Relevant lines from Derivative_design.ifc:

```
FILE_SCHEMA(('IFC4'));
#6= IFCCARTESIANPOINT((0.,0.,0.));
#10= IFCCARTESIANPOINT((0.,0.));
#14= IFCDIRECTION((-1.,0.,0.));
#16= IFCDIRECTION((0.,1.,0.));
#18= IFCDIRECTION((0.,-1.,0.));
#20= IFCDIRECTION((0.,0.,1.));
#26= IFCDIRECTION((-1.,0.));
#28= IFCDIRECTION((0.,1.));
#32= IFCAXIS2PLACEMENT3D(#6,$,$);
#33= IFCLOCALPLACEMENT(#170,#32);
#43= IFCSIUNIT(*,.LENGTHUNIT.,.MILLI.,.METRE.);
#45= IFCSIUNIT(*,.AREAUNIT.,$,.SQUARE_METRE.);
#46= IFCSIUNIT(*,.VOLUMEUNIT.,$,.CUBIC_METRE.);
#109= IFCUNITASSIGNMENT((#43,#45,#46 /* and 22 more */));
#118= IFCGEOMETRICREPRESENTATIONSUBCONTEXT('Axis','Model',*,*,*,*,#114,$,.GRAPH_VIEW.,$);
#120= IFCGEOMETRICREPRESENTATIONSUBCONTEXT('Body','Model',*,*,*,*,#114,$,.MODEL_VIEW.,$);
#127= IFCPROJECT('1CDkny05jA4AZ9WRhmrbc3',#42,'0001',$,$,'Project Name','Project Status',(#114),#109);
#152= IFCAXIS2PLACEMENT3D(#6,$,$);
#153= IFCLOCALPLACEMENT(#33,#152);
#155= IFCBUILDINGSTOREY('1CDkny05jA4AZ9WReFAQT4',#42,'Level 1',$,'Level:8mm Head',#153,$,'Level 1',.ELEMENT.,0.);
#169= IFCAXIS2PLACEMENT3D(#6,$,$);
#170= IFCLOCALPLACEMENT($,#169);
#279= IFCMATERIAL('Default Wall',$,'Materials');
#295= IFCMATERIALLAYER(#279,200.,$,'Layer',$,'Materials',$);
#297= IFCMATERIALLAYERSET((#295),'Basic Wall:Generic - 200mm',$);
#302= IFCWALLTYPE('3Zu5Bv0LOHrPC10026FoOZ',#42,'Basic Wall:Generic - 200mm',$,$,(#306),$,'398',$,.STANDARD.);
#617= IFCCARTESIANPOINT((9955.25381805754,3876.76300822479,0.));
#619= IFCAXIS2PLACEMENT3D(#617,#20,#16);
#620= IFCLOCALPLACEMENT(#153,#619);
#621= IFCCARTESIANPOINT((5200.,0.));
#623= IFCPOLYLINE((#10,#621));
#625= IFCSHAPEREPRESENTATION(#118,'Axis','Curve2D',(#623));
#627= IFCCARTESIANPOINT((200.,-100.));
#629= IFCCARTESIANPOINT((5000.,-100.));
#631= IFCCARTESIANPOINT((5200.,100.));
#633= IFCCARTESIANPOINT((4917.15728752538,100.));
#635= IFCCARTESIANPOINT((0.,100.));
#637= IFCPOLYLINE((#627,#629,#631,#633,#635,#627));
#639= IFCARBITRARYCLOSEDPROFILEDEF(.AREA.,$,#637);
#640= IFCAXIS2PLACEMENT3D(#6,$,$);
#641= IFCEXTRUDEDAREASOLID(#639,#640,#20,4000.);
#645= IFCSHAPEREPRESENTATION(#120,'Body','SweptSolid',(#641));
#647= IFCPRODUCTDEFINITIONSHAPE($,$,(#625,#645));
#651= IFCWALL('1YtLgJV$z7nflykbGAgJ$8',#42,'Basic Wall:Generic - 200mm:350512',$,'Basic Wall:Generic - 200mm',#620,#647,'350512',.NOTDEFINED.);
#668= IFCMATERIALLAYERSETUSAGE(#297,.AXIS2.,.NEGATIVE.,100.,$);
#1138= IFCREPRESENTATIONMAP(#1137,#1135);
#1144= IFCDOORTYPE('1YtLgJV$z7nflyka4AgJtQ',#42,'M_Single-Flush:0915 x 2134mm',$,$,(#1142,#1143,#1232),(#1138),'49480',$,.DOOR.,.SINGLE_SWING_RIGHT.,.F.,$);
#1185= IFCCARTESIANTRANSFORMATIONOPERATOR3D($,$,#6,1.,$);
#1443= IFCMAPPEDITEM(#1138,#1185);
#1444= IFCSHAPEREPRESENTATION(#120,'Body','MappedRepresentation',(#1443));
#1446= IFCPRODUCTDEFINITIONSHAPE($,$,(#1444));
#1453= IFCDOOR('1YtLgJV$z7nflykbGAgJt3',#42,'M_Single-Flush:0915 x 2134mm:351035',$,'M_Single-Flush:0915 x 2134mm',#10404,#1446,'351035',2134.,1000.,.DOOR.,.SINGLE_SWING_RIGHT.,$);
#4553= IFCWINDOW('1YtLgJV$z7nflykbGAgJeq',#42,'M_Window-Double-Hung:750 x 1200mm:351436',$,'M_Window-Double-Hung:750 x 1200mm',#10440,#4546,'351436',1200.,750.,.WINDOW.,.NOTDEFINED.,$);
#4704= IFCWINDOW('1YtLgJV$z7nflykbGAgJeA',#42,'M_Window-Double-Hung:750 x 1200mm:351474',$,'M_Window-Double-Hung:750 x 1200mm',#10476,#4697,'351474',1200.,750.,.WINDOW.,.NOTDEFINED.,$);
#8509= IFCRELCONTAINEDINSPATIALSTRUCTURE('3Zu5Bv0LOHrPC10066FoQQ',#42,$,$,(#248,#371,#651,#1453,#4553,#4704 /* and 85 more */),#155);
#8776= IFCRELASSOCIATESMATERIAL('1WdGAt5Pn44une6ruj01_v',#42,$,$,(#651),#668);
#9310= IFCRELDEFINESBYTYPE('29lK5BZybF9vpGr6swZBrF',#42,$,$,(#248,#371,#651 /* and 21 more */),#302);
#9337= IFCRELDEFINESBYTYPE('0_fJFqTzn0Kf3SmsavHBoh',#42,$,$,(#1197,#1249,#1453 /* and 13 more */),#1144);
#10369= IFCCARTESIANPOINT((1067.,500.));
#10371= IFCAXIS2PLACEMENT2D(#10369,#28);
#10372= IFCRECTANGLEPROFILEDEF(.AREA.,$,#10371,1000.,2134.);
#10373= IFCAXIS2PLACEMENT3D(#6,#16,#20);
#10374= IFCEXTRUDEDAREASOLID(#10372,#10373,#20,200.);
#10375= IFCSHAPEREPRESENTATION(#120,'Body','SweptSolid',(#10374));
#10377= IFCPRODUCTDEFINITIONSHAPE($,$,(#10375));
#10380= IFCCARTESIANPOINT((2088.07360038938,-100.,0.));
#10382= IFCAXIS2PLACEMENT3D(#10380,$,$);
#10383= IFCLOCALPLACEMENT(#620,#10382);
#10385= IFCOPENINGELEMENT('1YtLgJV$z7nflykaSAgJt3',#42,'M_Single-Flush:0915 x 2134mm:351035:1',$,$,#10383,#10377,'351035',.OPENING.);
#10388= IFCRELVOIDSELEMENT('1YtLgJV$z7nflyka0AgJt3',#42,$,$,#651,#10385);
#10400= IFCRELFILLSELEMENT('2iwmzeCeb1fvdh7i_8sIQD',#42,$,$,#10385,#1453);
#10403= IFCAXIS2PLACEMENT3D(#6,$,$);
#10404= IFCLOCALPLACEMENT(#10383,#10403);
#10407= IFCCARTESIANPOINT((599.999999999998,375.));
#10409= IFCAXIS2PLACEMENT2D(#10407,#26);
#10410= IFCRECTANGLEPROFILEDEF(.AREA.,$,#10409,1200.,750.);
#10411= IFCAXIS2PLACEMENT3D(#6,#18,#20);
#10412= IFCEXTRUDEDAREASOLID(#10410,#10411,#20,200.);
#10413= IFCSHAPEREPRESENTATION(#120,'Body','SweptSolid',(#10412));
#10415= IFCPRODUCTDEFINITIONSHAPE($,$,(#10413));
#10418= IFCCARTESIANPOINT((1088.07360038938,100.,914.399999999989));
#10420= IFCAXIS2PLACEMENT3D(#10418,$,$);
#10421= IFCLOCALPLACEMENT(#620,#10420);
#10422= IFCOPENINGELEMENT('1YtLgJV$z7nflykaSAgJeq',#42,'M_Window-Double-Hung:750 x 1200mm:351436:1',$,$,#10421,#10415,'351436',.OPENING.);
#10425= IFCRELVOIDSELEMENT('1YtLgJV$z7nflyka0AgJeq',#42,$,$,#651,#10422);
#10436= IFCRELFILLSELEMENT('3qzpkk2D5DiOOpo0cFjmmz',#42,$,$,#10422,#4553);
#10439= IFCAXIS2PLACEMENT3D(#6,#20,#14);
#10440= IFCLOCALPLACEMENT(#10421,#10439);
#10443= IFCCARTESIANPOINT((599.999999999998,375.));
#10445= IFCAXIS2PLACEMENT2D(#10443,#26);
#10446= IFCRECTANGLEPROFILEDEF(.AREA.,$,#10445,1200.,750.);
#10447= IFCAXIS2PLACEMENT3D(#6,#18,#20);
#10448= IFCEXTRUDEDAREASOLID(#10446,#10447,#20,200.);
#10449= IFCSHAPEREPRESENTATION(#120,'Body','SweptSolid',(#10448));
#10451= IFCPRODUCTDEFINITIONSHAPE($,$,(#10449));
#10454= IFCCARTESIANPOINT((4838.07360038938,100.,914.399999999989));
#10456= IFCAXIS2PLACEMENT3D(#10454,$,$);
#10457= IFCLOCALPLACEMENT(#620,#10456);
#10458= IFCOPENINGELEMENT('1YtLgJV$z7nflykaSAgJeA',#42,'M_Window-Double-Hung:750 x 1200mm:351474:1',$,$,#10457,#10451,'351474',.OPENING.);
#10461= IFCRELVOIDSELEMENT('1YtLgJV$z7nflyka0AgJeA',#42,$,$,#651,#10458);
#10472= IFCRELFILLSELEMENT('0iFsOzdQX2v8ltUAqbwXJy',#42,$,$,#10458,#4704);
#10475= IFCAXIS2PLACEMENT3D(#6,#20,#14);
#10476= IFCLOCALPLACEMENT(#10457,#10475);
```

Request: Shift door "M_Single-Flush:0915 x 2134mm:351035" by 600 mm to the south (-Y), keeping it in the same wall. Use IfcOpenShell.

```python
import ifcopenshell
import ifcopenshell.api.geometry
import ifcopenshell.util.placement

model = ifcopenshell.open("Derivative_design.ifc")

door = model.by_guid("1YtLgJV$z7nflykbGAgJt3")
opening = door.FillsVoids[0].RelatingOpeningElement
wall = opening.VoidsElements[0].RelatingBuildingElement

wall_matrix = ifcopenshell.util.placement.get_local_placement(wall.ObjectPlacement)
shift = wall_matrix[:3, 0] * -600.0
before = ifcopenshell.util.placement.get_local_placement(door.ObjectPlacement)[:3, 3].copy()

# The door is placed relative to its opening, so it follows when the opening moves.
matrix = ifcopenshell.util.placement.get_local_placement(opening.ObjectPlacement)
matrix[:3, 3] += shift
ifcopenshell.api.geometry.edit_object_placement(
    model, product=opening, matrix=matrix, is_si=False, should_transform_children=True
)

after = ifcopenshell.util.placement.get_local_placement(door.ObjectPlacement)[:3, 3]
print("door moved by", (after - before).round(3) + 0.0)

model.write("Derivative_design-out.ifc")
```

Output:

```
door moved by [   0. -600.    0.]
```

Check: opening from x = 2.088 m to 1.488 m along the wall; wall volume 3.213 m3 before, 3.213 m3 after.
